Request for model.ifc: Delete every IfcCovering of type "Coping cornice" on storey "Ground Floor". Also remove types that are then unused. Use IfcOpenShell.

First a look at what the model holds.

```python
import ifcopenshell
import ifcopenshell.util.element

model = ifcopenshell.open("model.ifc")
print(model.schema)
storey = next(s for s in model.by_type("IfcBuildingStorey") if s.Name == "Ground Floor")
coverings = [e for e in ifcopenshell.util.element.get_decomposition(storey) if e.is_a("IfcCovering")]
seen = {}
for e in coverings:
    element_type = ifcopenshell.util.element.get_type(e)
    name = element_type.Name if element_type not in (None, e) else None
    seen[name] = seen.get(name, 0) + 1
for name, count in sorted(seen.items(), key=str):
    print(count, "x", name)
```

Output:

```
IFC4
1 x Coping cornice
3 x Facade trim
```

```python
import ifcopenshell
import ifcopenshell.api.root
import ifcopenshell.util.element

model = ifcopenshell.open("model.ifc")

storey = next(s for s in model.by_type("IfcBuildingStorey") if s.Name == "Ground Floor")
coverings = [e for e in ifcopenshell.util.element.get_decomposition(storey) if e.is_a("IfcCovering")]
targets = [e for e in coverings if (t := ifcopenshell.util.element.get_type(e)) not in (None, e) and t.Name == "Coping cornice"]
types = {ifcopenshell.util.element.get_type(e) for e in targets} - {None, *targets}

for e in targets:
    ifcopenshell.api.root.remove_product(model, product=e)
print(len(targets), "removed")

unused = [t for t in types if not ifcopenshell.util.element.get_types(t)]
for t in unused:
    ifcopenshell.api.root.remove_product(model, product=t)
print(len(unused), "unused types removed")

model.write("model_updated.ifc")
```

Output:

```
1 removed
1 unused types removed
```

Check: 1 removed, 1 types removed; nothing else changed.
